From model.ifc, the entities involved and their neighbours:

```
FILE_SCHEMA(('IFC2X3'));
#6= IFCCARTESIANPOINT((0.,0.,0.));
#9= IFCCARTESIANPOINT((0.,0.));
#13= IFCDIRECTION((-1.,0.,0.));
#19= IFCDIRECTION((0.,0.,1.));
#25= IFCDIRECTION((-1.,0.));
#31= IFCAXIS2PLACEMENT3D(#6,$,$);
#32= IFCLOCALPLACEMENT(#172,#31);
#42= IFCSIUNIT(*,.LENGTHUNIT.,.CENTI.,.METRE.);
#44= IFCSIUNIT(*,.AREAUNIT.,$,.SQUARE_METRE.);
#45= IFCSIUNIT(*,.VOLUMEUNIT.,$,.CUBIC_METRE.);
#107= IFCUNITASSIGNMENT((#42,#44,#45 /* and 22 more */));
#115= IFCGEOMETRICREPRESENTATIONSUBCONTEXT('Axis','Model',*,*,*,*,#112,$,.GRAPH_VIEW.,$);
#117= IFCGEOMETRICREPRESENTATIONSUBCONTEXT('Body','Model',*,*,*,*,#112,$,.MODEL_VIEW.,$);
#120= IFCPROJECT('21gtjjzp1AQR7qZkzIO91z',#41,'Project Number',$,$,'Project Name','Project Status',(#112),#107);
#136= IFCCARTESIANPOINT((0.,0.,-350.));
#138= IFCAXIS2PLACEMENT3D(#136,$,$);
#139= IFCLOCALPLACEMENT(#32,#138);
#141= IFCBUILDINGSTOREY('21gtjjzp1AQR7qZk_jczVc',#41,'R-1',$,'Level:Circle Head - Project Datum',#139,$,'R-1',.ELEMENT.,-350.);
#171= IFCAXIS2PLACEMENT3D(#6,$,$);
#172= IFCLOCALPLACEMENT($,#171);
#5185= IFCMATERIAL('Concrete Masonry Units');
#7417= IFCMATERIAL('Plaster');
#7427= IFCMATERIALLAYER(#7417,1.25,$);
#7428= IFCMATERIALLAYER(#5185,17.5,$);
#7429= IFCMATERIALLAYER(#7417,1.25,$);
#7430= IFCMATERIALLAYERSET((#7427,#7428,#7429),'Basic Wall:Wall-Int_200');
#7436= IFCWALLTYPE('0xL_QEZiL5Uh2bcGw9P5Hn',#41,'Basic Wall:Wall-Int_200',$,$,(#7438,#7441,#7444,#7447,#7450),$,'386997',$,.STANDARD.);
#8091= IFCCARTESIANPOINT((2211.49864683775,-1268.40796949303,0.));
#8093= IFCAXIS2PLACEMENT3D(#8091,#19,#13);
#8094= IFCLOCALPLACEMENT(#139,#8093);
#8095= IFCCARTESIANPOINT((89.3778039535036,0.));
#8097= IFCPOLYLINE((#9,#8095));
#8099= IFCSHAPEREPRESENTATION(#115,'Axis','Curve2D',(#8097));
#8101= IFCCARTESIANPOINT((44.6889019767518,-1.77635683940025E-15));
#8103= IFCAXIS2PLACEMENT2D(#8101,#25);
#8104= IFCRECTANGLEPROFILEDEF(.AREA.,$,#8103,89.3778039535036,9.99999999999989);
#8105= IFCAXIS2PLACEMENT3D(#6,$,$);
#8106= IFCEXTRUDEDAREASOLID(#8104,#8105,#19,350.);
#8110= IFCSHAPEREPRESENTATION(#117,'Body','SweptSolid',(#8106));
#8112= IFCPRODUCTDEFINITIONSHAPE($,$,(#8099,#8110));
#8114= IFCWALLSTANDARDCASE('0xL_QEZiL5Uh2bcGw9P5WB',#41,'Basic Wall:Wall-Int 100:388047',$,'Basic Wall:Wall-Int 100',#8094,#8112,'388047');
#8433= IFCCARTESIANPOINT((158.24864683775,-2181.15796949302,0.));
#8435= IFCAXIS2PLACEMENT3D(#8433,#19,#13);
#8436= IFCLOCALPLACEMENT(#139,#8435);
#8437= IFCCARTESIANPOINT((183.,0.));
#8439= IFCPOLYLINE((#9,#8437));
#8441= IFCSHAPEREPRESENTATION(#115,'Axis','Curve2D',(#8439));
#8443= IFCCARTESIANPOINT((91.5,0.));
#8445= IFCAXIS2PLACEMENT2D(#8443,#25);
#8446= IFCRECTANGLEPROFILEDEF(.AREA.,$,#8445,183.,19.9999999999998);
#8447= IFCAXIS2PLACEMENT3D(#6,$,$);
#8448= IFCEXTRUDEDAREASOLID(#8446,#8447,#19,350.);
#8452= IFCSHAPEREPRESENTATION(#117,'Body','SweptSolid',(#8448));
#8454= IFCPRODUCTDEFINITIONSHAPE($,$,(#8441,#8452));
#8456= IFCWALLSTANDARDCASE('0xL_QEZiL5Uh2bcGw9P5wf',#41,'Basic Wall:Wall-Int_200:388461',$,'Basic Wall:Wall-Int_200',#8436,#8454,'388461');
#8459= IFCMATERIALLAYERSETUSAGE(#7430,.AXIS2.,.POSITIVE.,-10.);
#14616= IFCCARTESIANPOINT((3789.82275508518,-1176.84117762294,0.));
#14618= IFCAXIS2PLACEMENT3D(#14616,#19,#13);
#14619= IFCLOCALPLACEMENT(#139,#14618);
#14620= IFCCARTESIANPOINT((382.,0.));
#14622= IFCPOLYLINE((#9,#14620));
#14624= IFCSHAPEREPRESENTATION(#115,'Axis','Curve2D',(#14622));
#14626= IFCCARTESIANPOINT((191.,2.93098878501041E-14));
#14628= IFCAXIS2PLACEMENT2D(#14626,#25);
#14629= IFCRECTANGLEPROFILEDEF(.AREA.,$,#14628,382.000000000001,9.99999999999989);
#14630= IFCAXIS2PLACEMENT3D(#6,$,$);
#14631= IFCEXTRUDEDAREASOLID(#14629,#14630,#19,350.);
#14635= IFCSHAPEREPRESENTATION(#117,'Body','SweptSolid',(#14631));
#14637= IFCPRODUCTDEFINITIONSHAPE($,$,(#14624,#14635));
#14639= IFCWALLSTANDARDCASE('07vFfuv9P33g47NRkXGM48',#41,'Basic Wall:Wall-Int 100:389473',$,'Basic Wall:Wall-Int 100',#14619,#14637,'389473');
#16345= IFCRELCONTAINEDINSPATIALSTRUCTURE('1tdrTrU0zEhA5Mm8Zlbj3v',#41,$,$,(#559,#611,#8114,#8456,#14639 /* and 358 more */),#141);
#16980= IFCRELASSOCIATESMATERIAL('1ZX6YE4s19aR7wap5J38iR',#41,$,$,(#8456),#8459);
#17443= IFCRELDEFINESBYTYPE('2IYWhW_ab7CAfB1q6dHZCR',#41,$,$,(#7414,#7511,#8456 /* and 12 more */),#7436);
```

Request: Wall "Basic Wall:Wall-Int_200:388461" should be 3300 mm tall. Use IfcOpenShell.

```python
import ifcopenshell
import ifcopenshell.geom
import ifcopenshell.util.representation
import ifcopenshell.util.shape
import ifcopenshell.util.unit

model = ifcopenshell.open("model.ifc")
unit_scale = ifcopenshell.util.unit.calculate_unit_scale(model)
settings = ifcopenshell.geom.settings()


def volume(element):
    """Net volume in cubic metres, openings subtracted."""
    shape = ifcopenshell.geom.create_shape(settings, element)
    return ifcopenshell.util.shape.get_volume(shape.geometry)


wall = model.by_id(8456)
before = volume(wall)

body = ifcopenshell.util.representation.get_representation(wall, "Model", "Body")
solid = body.Items[0]
old_height = solid.Depth
solid.Depth = 3.3 / unit_scale
after = volume(wall)

print(f"height {old_height:g} -> {solid.Depth:g}, volume {before:.3f} -> {after:.3f} m3")

model.write("model_updated.ifc")
```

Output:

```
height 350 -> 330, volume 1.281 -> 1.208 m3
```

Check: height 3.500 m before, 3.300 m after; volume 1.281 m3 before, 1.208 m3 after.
